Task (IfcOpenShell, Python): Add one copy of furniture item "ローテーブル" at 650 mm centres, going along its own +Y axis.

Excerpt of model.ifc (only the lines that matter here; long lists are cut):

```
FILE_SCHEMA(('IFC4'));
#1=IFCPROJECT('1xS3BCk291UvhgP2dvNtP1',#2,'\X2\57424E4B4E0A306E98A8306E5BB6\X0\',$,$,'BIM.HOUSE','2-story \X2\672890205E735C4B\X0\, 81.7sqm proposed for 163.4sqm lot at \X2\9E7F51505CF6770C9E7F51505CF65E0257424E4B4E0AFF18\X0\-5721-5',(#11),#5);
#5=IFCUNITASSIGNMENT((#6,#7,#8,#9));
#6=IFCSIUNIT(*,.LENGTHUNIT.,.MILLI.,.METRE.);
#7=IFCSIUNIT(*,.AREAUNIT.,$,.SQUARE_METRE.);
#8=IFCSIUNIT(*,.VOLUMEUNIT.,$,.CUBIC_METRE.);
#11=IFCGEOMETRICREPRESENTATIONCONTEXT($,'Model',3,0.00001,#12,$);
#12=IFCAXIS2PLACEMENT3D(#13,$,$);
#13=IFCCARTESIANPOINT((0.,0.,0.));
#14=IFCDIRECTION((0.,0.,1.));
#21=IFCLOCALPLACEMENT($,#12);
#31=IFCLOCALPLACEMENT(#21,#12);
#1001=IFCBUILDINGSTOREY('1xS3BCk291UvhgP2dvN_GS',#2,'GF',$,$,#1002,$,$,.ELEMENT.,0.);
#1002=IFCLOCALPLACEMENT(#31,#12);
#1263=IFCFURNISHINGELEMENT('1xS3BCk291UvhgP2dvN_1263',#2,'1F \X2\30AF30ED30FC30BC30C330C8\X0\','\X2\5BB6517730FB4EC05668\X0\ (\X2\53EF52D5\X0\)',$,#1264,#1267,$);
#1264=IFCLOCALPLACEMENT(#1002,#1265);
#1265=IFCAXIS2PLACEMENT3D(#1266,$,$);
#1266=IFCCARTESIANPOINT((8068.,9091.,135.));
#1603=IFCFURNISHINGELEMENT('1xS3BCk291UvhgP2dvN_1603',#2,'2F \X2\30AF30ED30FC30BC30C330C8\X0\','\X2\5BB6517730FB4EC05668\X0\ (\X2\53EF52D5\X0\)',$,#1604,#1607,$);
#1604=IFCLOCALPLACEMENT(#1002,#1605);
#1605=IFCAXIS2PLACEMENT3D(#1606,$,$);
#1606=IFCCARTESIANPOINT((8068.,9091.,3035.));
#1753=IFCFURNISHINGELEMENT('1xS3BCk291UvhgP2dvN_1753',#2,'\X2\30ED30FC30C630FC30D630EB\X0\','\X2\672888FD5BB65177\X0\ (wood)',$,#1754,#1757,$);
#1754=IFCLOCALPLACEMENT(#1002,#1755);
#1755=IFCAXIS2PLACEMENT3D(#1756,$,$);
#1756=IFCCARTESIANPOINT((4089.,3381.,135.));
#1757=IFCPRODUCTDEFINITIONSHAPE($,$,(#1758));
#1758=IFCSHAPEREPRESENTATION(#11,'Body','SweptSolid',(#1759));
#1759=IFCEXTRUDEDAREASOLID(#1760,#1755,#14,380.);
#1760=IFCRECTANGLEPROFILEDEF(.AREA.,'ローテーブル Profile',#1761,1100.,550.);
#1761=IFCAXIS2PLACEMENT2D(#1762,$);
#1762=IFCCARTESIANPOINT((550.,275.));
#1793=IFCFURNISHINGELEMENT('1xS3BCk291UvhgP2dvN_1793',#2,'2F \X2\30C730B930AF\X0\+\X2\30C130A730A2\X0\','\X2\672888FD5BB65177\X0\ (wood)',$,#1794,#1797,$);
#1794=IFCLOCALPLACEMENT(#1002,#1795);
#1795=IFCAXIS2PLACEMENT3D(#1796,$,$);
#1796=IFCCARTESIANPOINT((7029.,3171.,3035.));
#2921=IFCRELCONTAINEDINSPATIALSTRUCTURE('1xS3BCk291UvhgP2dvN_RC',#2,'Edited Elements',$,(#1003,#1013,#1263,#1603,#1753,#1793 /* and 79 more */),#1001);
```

```python
import ifcopenshell
import ifcopenshell.api.geometry
import ifcopenshell.api.root
import ifcopenshell.util.element
import ifcopenshell.util.placement
import ifcopenshell.util.unit

model = ifcopenshell.open("model.ifc")
unit_scale = ifcopenshell.util.unit.calculate_unit_scale(model)


def reuse_history(source, copy):
    """copy_class also copies each property set's owner history, people and application; keep the originals."""
    for rel in copy.IsDefinedBy:
        if rel.is_a("IfcRelDefinesByProperties") and (history := rel.RelatingPropertyDefinition.OwnerHistory):
            rel.RelatingPropertyDefinition.OwnerHistory = source.OwnerHistory
            ifcopenshell.util.element.remove_deep2(model, history)


source = model.by_id(1753)
base = ifcopenshell.util.placement.get_local_placement(source.ObjectPlacement)
step = base[:3, 1] * 0.65 / unit_scale

for i in range(1, 2):
    copy = ifcopenshell.api.root.copy_class(model, product=source)
    copy.Representation = ifcopenshell.util.element.copy_deep(
        model, source.Representation, exclude=["IfcGeometricRepresentationContext", "IfcRepresentationMap"]
    )
    reuse_history(source, copy)
    matrix = base.copy()
    matrix[:3, 3] += i * step
    print("added at", matrix[:3, 3].round(3) + 0.0)
    ifcopenshell.api.geometry.edit_object_placement(model, product=copy, matrix=matrix, is_si=False)

model.write("model-out.ifc")
```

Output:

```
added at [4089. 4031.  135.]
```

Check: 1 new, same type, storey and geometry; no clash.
